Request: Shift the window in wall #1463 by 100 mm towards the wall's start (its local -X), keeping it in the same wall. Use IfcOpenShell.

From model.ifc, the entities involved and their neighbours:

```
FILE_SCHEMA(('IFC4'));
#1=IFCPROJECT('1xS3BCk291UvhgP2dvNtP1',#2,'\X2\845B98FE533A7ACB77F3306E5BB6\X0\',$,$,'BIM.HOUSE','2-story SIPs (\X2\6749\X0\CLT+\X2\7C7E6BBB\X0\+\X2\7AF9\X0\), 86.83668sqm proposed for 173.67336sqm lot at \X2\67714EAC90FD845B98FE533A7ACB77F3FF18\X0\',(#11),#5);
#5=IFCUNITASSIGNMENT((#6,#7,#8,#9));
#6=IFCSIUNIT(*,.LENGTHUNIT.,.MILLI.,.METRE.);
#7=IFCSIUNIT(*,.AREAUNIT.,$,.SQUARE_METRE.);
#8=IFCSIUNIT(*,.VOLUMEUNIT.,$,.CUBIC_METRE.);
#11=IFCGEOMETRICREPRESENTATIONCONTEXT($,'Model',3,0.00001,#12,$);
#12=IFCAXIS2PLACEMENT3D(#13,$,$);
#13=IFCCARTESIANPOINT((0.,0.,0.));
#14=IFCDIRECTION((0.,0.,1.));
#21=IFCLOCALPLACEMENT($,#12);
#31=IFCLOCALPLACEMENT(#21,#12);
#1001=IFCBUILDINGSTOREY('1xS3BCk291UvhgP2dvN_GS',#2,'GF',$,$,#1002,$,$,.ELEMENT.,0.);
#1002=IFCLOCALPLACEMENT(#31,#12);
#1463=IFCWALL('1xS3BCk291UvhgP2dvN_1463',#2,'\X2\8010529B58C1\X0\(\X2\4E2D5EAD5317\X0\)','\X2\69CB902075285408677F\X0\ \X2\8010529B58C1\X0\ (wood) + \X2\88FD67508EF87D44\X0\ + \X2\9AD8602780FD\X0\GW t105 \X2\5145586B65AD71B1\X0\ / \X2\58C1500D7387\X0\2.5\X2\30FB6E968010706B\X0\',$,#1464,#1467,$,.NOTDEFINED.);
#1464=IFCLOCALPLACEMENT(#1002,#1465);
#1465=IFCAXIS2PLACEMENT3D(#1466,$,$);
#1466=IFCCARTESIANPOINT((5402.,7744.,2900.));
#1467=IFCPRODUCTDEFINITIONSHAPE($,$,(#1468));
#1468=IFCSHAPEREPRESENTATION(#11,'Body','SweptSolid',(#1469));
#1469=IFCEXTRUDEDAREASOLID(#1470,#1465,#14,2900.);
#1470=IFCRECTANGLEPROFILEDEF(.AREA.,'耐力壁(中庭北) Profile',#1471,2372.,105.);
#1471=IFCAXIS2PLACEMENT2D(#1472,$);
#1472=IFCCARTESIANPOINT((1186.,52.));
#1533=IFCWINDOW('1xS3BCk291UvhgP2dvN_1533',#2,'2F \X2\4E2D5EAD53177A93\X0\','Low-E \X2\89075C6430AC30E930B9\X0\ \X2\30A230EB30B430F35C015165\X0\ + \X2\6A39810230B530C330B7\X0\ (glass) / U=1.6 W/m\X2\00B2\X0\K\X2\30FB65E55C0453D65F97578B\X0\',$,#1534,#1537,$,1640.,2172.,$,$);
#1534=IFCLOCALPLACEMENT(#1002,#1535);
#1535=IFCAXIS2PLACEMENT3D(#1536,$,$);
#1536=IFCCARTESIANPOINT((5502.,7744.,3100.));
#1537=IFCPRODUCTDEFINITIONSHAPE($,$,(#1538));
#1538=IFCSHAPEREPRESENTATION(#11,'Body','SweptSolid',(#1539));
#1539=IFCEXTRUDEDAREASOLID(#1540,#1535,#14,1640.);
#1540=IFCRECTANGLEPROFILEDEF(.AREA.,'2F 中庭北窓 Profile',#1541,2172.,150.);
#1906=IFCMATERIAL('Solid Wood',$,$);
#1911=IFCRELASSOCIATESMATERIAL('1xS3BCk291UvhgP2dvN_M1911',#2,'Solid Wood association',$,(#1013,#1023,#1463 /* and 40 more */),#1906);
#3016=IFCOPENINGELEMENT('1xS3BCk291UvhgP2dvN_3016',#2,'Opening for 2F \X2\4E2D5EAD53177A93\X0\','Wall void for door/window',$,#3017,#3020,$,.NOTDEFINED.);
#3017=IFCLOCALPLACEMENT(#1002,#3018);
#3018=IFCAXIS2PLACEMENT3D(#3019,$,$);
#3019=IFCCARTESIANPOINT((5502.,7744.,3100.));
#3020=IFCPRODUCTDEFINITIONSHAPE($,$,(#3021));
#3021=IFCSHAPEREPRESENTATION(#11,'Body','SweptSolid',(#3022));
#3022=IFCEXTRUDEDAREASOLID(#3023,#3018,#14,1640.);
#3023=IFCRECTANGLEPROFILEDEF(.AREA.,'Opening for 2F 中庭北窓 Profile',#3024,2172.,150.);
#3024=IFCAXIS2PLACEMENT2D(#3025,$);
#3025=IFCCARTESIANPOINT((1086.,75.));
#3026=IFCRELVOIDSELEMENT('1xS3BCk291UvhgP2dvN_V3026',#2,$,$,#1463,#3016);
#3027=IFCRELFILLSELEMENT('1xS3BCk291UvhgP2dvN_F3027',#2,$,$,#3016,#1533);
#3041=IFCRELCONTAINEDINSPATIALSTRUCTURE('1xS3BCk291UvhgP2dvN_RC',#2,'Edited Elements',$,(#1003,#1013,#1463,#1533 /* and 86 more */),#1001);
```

```python
import ifcopenshell
import ifcopenshell.api.geometry
import ifcopenshell.util.placement
import ifcopenshell.util.unit

model = ifcopenshell.open("model.ifc")
unit_scale = ifcopenshell.util.unit.calculate_unit_scale(model)

window = model.by_id(1533)
opening = window.FillsVoids[0].RelatingOpeningElement
wall = opening.VoidsElements[0].RelatingBuildingElement

wall_matrix = ifcopenshell.util.placement.get_local_placement(wall.ObjectPlacement)
shift = wall_matrix[:3, 0] * -0.1 / unit_scale
before = ifcopenshell.util.placement.get_local_placement(window.ObjectPlacement)[:3, 3].copy()

# The window is not placed relative to its opening, so move both.
for product in (opening, window):
    matrix = ifcopenshell.util.placement.get_local_placement(product.ObjectPlacement)
    matrix[:3, 3] += shift
    ifcopenshell.api.geometry.edit_object_placement(model, product=product, matrix=matrix, is_si=False)

after = ifcopenshell.util.placement.get_local_placement(window.ObjectPlacement)[:3, 3]
print("window moved by", (after - before).round(3) + 0.0)

model.write("model_v2.ifc")
```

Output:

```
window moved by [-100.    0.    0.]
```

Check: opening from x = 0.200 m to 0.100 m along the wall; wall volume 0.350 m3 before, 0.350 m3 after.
